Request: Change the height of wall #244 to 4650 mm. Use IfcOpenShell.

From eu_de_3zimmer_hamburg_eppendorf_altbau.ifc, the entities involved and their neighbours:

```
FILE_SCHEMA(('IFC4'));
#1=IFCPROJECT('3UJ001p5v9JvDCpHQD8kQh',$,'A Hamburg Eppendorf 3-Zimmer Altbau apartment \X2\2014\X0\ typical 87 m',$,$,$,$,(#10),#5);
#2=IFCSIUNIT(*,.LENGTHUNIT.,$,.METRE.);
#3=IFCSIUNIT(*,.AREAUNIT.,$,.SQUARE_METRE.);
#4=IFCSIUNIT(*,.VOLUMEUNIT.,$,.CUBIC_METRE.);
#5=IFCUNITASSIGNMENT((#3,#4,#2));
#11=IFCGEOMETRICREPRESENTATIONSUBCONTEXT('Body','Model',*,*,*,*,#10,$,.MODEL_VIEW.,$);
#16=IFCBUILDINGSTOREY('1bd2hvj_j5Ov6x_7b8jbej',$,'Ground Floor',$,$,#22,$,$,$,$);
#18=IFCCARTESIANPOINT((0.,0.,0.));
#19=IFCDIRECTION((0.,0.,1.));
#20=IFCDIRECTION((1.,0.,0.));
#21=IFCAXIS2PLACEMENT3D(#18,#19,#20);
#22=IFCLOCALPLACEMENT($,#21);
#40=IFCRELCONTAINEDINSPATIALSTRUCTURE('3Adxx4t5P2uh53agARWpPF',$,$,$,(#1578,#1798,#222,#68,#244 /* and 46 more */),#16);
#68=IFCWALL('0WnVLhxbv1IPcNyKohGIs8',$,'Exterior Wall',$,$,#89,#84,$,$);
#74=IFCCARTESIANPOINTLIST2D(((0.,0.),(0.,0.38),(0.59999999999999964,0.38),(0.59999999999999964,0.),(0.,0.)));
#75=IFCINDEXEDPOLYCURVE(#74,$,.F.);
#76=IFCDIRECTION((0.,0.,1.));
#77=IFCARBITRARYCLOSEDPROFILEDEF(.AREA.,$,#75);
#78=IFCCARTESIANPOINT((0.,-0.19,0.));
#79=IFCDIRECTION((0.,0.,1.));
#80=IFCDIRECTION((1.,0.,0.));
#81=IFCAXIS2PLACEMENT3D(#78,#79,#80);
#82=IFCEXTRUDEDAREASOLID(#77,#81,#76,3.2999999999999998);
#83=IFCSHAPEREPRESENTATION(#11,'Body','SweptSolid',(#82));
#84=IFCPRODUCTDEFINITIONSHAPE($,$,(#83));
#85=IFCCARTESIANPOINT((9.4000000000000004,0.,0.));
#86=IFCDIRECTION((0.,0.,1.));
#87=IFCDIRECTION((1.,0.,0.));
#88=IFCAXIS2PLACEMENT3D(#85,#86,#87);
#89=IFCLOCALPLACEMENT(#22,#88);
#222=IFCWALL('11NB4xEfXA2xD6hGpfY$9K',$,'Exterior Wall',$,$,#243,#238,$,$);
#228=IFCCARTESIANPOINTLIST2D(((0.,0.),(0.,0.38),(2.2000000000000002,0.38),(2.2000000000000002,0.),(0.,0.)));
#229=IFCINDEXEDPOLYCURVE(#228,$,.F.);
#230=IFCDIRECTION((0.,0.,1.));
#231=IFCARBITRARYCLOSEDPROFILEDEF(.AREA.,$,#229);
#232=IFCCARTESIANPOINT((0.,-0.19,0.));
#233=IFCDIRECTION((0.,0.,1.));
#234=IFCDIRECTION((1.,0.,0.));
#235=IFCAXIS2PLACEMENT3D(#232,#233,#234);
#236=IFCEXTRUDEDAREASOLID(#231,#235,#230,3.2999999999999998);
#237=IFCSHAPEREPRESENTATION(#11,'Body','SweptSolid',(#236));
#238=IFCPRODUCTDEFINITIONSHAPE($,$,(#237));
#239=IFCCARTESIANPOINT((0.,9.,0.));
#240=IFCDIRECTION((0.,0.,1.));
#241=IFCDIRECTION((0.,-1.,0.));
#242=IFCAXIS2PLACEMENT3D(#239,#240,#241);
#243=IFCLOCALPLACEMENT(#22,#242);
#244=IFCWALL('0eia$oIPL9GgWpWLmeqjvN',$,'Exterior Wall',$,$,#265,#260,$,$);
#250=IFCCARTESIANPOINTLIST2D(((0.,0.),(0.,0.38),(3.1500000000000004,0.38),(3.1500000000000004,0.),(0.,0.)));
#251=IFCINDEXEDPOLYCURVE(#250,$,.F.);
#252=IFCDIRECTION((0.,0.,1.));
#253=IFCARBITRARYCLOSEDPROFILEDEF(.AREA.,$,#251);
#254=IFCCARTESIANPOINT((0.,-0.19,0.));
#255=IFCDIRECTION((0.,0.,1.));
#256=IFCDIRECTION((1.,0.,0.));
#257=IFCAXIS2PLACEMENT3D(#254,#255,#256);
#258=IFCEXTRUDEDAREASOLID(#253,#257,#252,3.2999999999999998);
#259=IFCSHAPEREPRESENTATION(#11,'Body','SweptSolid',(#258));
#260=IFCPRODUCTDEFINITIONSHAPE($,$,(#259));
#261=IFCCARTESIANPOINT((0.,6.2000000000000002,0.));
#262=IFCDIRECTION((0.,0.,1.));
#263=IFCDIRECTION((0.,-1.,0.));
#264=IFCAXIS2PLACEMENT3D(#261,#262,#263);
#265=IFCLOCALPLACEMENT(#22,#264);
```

```python
import ifcopenshell
import ifcopenshell.geom
import ifcopenshell.util.representation
import ifcopenshell.util.shape
import ifcopenshell.util.unit

model = ifcopenshell.open("eu_de_3zimmer_hamburg_eppendorf_altbau.ifc")
unit_scale = ifcopenshell.util.unit.calculate_unit_scale(model)
settings = ifcopenshell.geom.settings()


def volume(element):
    """Net volume in cubic metres, openings subtracted."""
    shape = ifcopenshell.geom.create_shape(settings, element)
    return ifcopenshell.util.shape.get_volume(shape.geometry)


wall = model.by_guid("0eia$oIPL9GgWpWLmeqjvN")
before = volume(wall)

body = ifcopenshell.util.representation.get_representation(wall, "Model", "Body")
solid = body.Items[0]
old_height = solid.Depth
solid.Depth = 4.65 / unit_scale
after = volume(wall)

print(f"height {old_height:g} -> {solid.Depth:g}, volume {before:.3f} -> {after:.3f} m3")

model.write("eu_de_3zimmer_hamburg_eppendorf_altbau_rev.ifc")
```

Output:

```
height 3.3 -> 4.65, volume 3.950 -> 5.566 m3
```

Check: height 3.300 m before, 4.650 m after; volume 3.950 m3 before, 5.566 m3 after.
